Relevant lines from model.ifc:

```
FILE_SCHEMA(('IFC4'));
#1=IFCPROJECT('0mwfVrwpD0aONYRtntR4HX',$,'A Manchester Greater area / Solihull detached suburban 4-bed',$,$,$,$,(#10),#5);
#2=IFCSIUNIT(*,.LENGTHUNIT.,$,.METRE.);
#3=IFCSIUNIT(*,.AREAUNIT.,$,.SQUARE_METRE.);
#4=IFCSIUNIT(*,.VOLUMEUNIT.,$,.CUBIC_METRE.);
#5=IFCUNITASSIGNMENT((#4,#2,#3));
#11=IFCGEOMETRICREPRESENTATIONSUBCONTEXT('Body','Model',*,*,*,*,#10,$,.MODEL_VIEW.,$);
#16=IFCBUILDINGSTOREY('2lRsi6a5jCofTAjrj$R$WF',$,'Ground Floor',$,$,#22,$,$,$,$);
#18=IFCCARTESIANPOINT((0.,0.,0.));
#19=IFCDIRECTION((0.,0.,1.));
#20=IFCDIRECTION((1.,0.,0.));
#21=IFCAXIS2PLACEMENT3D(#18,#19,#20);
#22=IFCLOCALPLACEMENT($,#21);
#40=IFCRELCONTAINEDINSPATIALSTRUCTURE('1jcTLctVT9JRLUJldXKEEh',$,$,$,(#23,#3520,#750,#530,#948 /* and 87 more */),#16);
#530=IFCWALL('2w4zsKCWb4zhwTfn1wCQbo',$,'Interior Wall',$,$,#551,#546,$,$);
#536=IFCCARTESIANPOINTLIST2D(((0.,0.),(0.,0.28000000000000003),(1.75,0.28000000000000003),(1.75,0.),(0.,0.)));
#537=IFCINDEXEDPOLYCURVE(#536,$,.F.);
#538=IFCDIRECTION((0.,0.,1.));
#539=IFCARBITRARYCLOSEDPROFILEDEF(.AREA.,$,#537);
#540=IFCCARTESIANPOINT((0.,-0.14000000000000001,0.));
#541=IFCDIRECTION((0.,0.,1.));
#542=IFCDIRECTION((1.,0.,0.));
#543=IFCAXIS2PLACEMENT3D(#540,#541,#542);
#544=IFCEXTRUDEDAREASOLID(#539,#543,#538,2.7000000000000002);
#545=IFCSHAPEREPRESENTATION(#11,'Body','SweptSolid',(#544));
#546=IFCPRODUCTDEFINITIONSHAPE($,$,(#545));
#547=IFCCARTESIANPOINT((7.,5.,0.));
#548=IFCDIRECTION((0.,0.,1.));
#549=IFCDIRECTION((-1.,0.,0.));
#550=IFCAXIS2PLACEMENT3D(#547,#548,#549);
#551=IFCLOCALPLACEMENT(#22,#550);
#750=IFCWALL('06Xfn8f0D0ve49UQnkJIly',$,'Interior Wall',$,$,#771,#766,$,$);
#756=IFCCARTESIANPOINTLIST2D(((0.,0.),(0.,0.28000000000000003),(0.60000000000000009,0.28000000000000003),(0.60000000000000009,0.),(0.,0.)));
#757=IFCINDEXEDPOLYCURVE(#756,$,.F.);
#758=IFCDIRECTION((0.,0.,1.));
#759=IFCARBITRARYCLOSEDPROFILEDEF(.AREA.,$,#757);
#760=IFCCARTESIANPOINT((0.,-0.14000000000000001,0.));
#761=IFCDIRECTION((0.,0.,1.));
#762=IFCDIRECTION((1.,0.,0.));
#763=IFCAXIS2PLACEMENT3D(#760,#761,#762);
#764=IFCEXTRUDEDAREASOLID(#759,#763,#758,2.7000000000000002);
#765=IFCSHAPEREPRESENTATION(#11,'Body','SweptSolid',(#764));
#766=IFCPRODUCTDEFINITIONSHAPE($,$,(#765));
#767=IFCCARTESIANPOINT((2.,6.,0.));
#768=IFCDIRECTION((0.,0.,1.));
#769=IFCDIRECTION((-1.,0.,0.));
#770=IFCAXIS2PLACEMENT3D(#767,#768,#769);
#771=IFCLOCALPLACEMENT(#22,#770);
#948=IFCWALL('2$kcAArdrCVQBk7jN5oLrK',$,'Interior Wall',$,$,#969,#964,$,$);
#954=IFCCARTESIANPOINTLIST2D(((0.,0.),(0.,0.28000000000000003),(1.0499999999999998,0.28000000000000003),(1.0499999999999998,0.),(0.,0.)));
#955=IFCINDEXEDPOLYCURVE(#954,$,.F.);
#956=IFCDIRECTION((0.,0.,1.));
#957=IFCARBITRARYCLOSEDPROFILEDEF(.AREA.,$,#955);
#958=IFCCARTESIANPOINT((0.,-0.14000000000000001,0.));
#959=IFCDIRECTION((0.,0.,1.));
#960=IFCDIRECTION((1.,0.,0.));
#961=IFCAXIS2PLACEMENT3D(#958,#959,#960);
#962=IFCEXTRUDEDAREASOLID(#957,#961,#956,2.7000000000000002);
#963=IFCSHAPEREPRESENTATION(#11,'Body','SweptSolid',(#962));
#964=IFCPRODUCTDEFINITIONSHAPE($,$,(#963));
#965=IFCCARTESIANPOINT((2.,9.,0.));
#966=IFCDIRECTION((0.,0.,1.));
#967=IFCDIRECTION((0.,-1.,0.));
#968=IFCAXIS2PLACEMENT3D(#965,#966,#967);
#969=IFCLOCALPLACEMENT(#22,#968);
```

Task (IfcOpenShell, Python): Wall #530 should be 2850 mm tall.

```python
import ifcopenshell
import ifcopenshell.geom
import ifcopenshell.util.representation
import ifcopenshell.util.shape

model = ifcopenshell.open("model.ifc")
settings = ifcopenshell.geom.settings()


def volume(element):
    """Net volume in cubic metres, openings subtracted."""
    shape = ifcopenshell.geom.create_shape(settings, element)
    return ifcopenshell.util.shape.get_volume(shape.geometry)


wall = model.by_guid("2w4zsKCWb4zhwTfn1wCQbo")
before = volume(wall)

body = ifcopenshell.util.representation.get_representation(wall, "Model", "Body")
solid = body.Items[0]
old_height = solid.Depth
solid.Depth = 2.85
after = volume(wall)

print(f"height {old_height:g} -> {solid.Depth:g}, volume {before:.3f} -> {after:.3f} m3")

model.write("model_edited.ifc")
```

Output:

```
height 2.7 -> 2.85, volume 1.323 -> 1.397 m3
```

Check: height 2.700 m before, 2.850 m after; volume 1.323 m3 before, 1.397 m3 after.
